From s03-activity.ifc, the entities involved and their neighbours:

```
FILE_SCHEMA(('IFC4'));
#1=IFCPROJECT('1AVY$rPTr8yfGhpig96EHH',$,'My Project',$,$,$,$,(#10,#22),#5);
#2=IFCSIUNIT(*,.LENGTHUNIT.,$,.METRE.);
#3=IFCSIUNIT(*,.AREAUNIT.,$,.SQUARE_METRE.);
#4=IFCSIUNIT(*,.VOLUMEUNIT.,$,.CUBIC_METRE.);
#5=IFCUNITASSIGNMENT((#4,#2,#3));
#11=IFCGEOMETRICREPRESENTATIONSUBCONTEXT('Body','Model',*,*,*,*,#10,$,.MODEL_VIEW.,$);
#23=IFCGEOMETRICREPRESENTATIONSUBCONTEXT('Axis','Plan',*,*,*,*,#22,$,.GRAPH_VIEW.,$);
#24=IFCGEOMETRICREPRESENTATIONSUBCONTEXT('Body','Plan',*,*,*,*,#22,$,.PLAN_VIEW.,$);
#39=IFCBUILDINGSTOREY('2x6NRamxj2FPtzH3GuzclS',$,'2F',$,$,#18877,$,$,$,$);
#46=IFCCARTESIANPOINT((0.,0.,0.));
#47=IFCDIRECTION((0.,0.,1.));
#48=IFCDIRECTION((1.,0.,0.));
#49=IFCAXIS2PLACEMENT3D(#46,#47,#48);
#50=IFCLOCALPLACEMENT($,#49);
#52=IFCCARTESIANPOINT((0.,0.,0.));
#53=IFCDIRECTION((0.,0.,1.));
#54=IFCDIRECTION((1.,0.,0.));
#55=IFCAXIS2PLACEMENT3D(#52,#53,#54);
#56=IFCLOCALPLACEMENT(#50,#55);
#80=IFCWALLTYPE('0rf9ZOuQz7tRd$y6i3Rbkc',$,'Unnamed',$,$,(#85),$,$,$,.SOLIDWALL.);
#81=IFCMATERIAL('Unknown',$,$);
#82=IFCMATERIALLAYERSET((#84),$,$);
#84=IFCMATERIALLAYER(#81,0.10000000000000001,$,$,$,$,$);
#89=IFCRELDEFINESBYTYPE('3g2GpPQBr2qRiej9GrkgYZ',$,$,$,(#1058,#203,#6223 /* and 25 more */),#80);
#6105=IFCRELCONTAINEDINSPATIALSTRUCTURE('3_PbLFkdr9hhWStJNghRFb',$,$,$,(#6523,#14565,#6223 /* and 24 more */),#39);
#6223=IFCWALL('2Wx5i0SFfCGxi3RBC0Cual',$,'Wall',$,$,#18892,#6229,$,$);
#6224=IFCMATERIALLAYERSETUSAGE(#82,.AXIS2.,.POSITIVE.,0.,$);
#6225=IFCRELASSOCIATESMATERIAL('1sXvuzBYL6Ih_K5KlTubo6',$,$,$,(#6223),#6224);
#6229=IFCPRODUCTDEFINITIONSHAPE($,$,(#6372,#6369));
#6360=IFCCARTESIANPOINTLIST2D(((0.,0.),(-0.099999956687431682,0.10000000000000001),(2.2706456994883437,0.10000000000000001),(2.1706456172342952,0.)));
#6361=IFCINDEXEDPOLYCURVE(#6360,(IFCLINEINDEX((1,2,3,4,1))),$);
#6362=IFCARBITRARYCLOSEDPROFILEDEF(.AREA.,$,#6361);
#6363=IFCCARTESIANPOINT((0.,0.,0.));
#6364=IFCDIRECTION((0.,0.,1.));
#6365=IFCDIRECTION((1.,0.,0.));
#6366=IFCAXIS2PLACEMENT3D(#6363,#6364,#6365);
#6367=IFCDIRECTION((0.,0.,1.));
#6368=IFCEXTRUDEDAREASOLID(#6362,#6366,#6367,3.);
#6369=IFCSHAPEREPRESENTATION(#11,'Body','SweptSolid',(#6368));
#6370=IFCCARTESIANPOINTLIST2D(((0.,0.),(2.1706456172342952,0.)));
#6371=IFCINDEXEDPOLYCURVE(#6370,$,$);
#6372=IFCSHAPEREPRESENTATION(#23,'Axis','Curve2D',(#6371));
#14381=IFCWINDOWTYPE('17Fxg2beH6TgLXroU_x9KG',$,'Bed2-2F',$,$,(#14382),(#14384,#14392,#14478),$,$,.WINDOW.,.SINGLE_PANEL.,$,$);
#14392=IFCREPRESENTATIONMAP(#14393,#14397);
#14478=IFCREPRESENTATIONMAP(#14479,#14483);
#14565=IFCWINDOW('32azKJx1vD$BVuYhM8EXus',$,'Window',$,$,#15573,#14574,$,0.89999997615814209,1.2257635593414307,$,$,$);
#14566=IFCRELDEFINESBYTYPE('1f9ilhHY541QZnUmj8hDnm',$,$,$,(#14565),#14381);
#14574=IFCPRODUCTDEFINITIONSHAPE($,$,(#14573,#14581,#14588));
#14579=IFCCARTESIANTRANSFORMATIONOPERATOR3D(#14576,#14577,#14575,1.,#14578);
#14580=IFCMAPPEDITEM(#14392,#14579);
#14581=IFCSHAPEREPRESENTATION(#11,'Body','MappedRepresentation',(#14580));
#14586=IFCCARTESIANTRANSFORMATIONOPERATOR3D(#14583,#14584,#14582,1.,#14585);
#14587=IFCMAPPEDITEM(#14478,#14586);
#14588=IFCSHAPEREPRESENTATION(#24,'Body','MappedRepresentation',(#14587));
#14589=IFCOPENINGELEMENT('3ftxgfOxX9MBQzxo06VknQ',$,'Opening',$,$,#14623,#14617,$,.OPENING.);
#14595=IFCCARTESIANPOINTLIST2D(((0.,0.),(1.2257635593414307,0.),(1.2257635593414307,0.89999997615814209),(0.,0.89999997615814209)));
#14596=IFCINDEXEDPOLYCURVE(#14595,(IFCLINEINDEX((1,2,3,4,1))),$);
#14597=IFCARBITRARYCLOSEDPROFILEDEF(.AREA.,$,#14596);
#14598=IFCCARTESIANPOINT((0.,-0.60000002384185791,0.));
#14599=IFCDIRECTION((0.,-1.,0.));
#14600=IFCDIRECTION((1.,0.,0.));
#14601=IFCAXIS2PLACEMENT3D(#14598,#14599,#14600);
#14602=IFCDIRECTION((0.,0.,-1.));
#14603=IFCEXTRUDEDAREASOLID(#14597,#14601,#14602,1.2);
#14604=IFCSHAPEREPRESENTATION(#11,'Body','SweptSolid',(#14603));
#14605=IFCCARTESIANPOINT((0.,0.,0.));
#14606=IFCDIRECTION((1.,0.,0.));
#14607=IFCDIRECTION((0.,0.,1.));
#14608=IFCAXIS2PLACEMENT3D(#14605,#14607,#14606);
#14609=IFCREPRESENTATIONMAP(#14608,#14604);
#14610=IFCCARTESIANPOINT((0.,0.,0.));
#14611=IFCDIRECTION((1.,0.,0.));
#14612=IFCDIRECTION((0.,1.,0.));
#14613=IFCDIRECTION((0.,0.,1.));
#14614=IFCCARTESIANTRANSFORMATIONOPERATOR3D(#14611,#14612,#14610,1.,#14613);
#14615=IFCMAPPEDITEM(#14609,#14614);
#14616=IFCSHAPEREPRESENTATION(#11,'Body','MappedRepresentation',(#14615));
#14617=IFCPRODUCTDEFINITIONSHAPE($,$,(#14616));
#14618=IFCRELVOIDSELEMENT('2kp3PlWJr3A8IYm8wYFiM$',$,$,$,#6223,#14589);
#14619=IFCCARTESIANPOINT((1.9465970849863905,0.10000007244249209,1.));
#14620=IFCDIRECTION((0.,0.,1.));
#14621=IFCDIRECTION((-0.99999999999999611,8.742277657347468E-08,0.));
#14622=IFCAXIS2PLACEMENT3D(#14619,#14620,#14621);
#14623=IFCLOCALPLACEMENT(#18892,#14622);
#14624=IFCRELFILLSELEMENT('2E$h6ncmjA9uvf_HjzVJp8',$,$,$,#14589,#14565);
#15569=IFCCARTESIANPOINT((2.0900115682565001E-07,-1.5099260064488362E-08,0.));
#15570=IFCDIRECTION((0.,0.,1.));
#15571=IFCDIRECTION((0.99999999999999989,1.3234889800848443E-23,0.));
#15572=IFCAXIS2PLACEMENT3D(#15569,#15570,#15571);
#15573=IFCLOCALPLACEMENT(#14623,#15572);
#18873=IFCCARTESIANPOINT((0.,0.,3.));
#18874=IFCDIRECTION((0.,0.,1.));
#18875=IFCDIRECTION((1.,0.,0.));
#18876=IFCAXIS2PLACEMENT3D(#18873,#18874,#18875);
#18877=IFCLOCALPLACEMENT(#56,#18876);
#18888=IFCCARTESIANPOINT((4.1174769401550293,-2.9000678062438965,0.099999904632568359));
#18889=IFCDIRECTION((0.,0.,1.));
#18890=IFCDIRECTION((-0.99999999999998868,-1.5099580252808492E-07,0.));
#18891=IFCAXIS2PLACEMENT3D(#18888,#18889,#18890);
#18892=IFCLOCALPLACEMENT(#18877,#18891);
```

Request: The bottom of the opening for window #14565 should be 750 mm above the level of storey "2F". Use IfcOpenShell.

```python
import numpy as np
import ifcopenshell
import ifcopenshell.api.geometry
import ifcopenshell.geom
import ifcopenshell.util.element
import ifcopenshell.util.placement
import ifcopenshell.util.shape
import ifcopenshell.util.unit

model = ifcopenshell.open("s03-activity.ifc")
unit_scale = ifcopenshell.util.unit.calculate_unit_scale(model)

window = model.by_guid("32azKJx1vD$BVuYhM8EXus")
opening = window.FillsVoids[0].RelatingOpeningElement
storey = ifcopenshell.util.element.get_container(window, ifc_class="IfcBuildingStorey")
level = ifcopenshell.util.placement.get_local_placement(storey.ObjectPlacement)[2, 3]

# The opening's origin need not be at the sill, so measure its lowest point.
shape = ifcopenshell.geom.create_shape(ifcopenshell.geom.settings(), opening)
bottom = ifcopenshell.util.shape.get_shape_bottom_elevation(shape, shape.geometry) / unit_scale
dz = level + 0.75 - bottom

shift = np.array([0.0, 0.0, dz])
# The window is placed relative to its opening, so it follows when the opening moves.
matrix = ifcopenshell.util.placement.get_local_placement(opening.ObjectPlacement)
matrix[:3, 3] += shift
ifcopenshell.api.geometry.edit_object_placement(
    model, product=opening, matrix=matrix, is_si=False, should_transform_children=True
)

print(f"moved by {dz * unit_scale:+.3f} m")

model.write("s03-activity_updated.ifc")
```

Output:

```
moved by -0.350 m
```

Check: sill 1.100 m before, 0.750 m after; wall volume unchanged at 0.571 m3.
